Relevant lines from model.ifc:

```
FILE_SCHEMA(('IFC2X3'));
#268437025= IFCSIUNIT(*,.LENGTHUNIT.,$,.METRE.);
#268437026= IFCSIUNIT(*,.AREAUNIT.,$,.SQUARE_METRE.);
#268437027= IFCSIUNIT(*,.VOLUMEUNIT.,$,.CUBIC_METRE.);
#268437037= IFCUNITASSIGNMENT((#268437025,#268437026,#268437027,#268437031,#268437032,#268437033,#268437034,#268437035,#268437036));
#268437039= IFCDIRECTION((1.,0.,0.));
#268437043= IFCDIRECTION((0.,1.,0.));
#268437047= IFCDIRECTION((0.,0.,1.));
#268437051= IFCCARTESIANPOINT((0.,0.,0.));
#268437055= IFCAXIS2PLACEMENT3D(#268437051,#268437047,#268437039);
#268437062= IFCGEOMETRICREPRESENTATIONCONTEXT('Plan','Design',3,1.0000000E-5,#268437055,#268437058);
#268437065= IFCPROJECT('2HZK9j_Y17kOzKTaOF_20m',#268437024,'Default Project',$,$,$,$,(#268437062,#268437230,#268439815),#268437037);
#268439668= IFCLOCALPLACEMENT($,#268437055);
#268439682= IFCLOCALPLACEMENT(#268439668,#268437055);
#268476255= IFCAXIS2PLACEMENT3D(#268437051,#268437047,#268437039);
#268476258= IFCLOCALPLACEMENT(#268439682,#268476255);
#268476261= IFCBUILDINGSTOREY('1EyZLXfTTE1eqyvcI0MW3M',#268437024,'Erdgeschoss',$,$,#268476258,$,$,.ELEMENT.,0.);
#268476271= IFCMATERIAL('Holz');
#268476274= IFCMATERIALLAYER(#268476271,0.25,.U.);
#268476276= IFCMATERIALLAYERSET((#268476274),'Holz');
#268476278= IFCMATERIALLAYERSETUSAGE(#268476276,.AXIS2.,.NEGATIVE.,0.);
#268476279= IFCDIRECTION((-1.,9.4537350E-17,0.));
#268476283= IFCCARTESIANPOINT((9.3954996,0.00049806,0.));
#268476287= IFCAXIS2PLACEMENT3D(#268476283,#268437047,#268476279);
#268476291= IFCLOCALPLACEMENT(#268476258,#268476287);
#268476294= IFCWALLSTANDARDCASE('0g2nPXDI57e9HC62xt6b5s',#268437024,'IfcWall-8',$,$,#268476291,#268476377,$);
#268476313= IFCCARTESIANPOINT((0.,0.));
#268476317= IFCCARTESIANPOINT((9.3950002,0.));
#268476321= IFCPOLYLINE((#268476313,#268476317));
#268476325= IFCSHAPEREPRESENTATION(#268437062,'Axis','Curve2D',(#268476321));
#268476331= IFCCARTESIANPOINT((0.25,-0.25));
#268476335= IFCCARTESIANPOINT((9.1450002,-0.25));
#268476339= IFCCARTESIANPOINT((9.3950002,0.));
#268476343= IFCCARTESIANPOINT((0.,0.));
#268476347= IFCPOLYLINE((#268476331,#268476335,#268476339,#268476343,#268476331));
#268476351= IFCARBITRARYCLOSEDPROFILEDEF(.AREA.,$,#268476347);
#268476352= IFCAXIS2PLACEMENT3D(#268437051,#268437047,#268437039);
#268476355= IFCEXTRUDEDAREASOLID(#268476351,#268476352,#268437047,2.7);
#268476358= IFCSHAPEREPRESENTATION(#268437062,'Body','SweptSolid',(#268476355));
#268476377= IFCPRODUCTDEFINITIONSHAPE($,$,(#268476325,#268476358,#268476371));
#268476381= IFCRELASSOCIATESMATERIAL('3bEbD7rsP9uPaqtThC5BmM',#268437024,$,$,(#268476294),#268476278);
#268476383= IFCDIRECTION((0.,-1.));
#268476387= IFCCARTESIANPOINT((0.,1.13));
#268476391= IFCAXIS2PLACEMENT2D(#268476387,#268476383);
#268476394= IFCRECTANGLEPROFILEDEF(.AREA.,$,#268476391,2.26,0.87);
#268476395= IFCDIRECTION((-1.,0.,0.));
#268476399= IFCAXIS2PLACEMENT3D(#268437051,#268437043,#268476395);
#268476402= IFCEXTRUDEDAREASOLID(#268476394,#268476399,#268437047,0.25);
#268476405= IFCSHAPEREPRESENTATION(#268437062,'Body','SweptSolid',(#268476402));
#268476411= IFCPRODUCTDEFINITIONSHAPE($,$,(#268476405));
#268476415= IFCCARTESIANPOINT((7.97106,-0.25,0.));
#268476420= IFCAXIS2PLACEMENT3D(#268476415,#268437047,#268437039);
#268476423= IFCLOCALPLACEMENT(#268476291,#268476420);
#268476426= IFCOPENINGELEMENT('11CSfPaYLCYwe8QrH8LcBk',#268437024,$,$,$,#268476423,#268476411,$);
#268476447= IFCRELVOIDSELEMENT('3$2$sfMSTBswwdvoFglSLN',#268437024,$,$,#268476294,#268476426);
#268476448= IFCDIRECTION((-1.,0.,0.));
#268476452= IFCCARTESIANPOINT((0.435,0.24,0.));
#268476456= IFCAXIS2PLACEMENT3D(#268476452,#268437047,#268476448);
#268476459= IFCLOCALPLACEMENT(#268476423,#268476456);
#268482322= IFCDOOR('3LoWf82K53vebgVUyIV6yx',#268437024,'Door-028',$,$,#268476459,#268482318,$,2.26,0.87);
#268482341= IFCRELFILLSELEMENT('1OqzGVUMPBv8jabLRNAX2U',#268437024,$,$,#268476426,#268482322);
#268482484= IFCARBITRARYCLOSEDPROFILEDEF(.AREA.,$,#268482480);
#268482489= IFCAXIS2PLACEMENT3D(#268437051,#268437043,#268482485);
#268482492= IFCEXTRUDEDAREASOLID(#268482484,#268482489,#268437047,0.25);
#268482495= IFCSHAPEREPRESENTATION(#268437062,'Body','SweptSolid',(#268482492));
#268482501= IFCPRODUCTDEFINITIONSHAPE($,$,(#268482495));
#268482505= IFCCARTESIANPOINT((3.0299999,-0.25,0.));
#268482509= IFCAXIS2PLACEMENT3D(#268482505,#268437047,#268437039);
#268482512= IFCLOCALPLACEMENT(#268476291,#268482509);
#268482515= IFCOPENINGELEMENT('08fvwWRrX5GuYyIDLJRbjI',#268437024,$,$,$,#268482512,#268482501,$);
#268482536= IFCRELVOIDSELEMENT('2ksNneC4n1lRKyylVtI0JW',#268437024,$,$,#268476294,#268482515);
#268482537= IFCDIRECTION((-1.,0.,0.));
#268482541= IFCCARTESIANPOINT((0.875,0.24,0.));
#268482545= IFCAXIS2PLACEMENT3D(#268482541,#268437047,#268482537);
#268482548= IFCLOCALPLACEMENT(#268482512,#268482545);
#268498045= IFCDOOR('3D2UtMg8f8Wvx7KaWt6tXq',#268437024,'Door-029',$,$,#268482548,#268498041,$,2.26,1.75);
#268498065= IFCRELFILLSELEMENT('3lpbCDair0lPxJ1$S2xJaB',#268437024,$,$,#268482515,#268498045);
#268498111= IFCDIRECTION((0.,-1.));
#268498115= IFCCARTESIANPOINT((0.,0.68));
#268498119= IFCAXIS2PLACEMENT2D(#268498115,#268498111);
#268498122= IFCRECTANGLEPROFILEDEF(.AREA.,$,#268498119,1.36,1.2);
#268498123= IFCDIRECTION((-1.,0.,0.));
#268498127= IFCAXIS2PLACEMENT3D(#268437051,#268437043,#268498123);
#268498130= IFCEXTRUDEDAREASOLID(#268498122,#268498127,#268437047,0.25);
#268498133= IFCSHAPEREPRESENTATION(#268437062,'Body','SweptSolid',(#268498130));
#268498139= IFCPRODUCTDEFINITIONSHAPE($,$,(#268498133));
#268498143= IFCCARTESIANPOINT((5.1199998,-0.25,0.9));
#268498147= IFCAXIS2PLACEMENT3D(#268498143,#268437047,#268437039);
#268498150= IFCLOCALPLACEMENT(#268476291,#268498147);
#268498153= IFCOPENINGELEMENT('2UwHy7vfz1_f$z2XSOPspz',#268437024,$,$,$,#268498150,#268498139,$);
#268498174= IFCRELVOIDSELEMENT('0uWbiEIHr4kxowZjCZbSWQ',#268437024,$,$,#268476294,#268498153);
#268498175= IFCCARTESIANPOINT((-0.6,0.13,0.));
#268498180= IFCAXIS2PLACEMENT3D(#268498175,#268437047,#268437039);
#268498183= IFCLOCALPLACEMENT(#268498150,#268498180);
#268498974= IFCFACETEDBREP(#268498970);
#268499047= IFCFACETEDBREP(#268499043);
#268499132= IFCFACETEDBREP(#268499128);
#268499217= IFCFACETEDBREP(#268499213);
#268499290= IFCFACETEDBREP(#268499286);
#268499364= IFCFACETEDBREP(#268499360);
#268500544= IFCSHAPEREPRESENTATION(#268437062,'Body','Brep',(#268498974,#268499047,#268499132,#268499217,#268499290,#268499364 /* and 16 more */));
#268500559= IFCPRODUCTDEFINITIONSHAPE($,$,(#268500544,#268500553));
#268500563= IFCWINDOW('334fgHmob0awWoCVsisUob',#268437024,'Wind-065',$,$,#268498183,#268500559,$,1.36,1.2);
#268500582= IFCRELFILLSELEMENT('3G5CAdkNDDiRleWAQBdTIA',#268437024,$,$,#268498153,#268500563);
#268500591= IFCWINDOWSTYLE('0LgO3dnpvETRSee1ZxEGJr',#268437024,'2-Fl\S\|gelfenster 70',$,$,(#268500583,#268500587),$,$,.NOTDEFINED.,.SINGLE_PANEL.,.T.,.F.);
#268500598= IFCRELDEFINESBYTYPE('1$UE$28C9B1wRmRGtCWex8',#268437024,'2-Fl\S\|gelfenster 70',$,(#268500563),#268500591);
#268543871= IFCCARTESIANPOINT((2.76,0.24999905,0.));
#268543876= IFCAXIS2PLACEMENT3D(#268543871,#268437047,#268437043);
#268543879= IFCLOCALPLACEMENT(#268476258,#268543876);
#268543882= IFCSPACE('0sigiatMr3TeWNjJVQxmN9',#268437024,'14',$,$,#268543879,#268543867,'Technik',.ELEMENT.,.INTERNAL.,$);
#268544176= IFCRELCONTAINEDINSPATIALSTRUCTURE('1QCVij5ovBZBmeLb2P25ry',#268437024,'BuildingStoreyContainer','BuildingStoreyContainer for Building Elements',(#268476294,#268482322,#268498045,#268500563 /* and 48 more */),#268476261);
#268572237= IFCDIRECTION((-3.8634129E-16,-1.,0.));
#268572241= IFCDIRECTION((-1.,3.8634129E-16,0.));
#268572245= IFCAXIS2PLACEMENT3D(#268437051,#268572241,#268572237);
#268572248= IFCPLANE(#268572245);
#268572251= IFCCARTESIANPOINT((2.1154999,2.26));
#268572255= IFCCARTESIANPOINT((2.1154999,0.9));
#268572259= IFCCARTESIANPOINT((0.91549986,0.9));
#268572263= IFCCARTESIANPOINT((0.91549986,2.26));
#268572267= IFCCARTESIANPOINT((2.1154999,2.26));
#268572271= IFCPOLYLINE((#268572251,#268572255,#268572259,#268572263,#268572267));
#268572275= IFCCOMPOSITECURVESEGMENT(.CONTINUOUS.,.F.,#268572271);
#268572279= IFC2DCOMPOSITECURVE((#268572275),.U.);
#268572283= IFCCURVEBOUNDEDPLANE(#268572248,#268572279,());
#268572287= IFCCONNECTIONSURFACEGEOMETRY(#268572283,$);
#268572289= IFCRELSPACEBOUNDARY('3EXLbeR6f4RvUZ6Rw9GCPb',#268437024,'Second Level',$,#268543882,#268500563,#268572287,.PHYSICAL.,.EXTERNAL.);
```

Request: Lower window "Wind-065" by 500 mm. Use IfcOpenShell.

```python
import numpy as np
import ifcopenshell
import ifcopenshell.api.geometry
import ifcopenshell.util.placement
import ifcopenshell.util.unit

model = ifcopenshell.open("model.ifc")
unit_scale = ifcopenshell.util.unit.calculate_unit_scale(model)

window = model.by_guid("334fgHmob0awWoCVsisUob")
opening = window.FillsVoids[0].RelatingOpeningElement
dz = -0.5

shift = np.array([0.0, 0.0, dz])
# The window is placed relative to its opening, so it follows when the opening moves.
matrix = ifcopenshell.util.placement.get_local_placement(opening.ObjectPlacement)
matrix[:3, 3] += shift
ifcopenshell.api.geometry.edit_object_placement(
    model, product=opening, matrix=matrix, is_si=False, should_transform_children=True
)

# Space boundary surfaces are stored in each space's coordinates; move them too.
for rel in window.ProvidesBoundaries:
    if not rel.ConnectionGeometry:
        continue
    surface = rel.ConnectionGeometry.SurfaceOnRelatingElement.BasisSurface
    space_matrix = ifcopenshell.util.placement.get_local_placement(rel.RelatingSpace.ObjectPlacement)
    point = np.array(surface.Position.Location.Coordinates) + space_matrix[:3, :3].T @ shift
    surface.Position = model.createIfcAxis2Placement3D(
        model.createIfcCartesianPoint(point.tolist()), surface.Position.Axis, surface.Position.RefDirection
    )

print(f"moved by {dz * unit_scale:+.3f} m")

model.write("model_rev.ifc")
```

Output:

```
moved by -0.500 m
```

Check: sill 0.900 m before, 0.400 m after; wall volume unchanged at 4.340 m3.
